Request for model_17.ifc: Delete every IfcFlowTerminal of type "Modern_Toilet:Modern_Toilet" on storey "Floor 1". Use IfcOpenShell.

First a look at what the model holds.

```python
import ifcopenshell
import ifcopenshell.util.element

model = ifcopenshell.open("model_17.ifc")
print(model.schema)
storey = next(s for s in model.by_type("IfcBuildingStorey") if s.Name == "Floor 1")
terminals = [e for e in ifcopenshell.util.element.get_decomposition(storey) if e.is_a("IfcFlowTerminal")]
seen = {}
for e in terminals:
    element_type = ifcopenshell.util.element.get_type(e)
    name = element_type.Name if element_type not in (None, e) else None
    seen[name] = seen.get(name, 0) + 1
for name, count in sorted(seen.items(), key=str):
    print(count, "x", name)
```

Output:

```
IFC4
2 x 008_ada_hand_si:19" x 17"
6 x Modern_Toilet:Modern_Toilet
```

```python
import ifcopenshell
import ifcopenshell.api.root
import ifcopenshell.util.element

model = ifcopenshell.open("model_17.ifc")

storey = next(s for s in model.by_type("IfcBuildingStorey") if s.Name == "Floor 1")
terminals = [e for e in ifcopenshell.util.element.get_decomposition(storey) if e.is_a("IfcFlowTerminal")]
targets = [e for e in terminals if (t := ifcopenshell.util.element.get_type(e)) not in (None, e) and t.Name == "Modern_Toilet:Modern_Toilet"]

for e in targets:
    ifcopenshell.api.root.remove_product(model, product=e)
print(len(targets), "removed")

model.write("model_17_rev.ifc")
```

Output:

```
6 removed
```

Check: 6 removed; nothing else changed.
